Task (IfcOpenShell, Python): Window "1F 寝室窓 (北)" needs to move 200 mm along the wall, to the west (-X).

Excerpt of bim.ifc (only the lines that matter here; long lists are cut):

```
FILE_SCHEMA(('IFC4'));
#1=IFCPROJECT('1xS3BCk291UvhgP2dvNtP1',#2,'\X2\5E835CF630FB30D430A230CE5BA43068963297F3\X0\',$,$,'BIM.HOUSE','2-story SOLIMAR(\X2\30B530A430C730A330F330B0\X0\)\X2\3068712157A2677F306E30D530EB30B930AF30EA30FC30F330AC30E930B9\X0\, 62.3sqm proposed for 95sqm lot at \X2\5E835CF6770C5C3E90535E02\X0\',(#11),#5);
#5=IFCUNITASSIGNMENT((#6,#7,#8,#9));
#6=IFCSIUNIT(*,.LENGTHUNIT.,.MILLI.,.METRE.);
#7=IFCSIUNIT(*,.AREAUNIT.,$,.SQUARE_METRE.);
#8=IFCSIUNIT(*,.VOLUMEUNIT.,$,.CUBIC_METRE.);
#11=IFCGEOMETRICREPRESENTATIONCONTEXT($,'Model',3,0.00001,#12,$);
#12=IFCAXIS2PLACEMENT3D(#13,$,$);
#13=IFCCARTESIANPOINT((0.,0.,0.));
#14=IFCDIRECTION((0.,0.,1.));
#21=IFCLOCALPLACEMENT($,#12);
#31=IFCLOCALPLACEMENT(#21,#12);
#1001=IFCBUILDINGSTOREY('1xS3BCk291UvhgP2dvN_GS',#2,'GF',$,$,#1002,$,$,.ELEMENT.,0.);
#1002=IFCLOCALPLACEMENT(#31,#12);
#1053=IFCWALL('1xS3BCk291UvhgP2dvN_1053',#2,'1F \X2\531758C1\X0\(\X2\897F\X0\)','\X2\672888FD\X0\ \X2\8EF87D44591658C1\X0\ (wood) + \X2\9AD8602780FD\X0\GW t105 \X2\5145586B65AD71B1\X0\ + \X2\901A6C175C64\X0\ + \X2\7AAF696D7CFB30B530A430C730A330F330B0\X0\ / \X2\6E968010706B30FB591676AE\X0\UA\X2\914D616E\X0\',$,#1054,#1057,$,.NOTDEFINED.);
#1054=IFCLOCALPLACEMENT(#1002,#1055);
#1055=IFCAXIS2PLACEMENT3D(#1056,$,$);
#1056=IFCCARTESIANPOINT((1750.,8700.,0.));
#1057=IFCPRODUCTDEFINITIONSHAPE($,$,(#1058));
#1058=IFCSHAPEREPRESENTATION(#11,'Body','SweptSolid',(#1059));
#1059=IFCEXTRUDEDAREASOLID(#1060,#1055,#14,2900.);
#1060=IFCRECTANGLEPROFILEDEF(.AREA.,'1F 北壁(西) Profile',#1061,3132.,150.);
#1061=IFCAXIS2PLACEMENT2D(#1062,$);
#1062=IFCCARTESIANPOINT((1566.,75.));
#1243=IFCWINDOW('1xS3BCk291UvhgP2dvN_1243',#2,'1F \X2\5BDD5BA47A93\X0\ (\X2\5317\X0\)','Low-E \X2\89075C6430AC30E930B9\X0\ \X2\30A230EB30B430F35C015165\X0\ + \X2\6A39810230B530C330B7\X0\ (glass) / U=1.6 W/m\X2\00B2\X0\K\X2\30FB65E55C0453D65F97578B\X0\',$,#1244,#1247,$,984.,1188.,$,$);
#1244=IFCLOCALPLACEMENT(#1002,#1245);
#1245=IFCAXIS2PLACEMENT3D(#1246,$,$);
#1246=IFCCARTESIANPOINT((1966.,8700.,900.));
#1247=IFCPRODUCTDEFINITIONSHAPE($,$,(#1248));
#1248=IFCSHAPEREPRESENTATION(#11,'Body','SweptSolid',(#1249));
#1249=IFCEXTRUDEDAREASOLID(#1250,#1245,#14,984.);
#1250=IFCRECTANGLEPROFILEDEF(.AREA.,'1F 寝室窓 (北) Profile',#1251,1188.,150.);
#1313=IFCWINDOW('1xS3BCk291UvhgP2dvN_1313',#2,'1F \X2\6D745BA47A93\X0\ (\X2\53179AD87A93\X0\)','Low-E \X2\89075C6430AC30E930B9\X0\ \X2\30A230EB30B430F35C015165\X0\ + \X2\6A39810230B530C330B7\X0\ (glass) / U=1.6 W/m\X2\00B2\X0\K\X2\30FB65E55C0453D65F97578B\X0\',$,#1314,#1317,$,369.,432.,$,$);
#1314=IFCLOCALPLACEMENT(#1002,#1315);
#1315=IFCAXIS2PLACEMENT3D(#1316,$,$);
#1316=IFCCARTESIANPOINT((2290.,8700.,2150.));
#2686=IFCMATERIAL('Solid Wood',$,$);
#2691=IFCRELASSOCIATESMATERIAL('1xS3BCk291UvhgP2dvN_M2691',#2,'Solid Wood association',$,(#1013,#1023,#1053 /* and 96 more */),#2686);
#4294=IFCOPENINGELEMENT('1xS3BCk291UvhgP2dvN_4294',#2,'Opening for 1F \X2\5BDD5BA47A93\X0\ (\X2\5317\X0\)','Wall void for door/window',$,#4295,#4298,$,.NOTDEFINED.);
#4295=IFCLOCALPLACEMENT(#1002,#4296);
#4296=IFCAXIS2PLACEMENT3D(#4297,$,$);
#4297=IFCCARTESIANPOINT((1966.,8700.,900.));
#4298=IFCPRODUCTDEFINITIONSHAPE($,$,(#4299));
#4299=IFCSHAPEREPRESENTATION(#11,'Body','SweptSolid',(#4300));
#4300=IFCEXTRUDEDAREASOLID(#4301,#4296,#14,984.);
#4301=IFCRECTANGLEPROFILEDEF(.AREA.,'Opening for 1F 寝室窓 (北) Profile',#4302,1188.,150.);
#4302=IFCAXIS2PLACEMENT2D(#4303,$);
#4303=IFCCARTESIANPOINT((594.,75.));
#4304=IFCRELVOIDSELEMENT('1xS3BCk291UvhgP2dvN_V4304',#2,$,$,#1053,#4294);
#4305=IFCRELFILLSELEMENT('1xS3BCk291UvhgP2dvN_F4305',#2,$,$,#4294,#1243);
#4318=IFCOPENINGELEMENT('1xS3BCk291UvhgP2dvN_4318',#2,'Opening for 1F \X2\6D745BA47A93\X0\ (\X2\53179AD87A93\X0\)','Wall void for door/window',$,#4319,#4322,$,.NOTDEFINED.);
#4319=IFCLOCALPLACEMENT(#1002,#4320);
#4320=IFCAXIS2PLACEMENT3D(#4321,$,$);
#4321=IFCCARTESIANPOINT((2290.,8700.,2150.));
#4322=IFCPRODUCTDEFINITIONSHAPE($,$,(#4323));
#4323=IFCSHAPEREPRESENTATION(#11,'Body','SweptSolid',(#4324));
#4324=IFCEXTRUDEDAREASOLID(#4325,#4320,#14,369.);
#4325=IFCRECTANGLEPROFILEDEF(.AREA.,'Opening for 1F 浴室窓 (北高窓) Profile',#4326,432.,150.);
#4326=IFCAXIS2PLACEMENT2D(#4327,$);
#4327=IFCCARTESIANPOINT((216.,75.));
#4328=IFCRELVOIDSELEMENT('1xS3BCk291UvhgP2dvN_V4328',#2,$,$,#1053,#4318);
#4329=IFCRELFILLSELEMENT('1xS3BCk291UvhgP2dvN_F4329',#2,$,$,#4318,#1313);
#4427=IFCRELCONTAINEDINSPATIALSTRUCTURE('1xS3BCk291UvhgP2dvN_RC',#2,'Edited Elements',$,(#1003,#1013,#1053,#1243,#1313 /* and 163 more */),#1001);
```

```python
import ifcopenshell
import ifcopenshell.api.geometry
import ifcopenshell.util.placement

model = ifcopenshell.open("bim.ifc")

window = model.by_guid("1xS3BCk291UvhgP2dvN_1243")
opening = window.FillsVoids[0].RelatingOpeningElement
wall = opening.VoidsElements[0].RelatingBuildingElement

wall_matrix = ifcopenshell.util.placement.get_local_placement(wall.ObjectPlacement)
shift = wall_matrix[:3, 0] * -200.0
before = ifcopenshell.util.placement.get_local_placement(window.ObjectPlacement)[:3, 3].copy()

# The window is not placed relative to its opening, so move both.
for product in (opening, window):
    matrix = ifcopenshell.util.placement.get_local_placement(product.ObjectPlacement)
    matrix[:3, 3] += shift
    ifcopenshell.api.geometry.edit_object_placement(model, product=product, matrix=matrix, is_si=False)

after = ifcopenshell.util.placement.get_local_placement(window.ObjectPlacement)[:3, 3]
print("window moved by", (after - before).round(3) + 0.0)

model.write("bim-out.ifc")
```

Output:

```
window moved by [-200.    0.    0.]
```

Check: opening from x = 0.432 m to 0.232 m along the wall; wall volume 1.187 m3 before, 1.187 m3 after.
